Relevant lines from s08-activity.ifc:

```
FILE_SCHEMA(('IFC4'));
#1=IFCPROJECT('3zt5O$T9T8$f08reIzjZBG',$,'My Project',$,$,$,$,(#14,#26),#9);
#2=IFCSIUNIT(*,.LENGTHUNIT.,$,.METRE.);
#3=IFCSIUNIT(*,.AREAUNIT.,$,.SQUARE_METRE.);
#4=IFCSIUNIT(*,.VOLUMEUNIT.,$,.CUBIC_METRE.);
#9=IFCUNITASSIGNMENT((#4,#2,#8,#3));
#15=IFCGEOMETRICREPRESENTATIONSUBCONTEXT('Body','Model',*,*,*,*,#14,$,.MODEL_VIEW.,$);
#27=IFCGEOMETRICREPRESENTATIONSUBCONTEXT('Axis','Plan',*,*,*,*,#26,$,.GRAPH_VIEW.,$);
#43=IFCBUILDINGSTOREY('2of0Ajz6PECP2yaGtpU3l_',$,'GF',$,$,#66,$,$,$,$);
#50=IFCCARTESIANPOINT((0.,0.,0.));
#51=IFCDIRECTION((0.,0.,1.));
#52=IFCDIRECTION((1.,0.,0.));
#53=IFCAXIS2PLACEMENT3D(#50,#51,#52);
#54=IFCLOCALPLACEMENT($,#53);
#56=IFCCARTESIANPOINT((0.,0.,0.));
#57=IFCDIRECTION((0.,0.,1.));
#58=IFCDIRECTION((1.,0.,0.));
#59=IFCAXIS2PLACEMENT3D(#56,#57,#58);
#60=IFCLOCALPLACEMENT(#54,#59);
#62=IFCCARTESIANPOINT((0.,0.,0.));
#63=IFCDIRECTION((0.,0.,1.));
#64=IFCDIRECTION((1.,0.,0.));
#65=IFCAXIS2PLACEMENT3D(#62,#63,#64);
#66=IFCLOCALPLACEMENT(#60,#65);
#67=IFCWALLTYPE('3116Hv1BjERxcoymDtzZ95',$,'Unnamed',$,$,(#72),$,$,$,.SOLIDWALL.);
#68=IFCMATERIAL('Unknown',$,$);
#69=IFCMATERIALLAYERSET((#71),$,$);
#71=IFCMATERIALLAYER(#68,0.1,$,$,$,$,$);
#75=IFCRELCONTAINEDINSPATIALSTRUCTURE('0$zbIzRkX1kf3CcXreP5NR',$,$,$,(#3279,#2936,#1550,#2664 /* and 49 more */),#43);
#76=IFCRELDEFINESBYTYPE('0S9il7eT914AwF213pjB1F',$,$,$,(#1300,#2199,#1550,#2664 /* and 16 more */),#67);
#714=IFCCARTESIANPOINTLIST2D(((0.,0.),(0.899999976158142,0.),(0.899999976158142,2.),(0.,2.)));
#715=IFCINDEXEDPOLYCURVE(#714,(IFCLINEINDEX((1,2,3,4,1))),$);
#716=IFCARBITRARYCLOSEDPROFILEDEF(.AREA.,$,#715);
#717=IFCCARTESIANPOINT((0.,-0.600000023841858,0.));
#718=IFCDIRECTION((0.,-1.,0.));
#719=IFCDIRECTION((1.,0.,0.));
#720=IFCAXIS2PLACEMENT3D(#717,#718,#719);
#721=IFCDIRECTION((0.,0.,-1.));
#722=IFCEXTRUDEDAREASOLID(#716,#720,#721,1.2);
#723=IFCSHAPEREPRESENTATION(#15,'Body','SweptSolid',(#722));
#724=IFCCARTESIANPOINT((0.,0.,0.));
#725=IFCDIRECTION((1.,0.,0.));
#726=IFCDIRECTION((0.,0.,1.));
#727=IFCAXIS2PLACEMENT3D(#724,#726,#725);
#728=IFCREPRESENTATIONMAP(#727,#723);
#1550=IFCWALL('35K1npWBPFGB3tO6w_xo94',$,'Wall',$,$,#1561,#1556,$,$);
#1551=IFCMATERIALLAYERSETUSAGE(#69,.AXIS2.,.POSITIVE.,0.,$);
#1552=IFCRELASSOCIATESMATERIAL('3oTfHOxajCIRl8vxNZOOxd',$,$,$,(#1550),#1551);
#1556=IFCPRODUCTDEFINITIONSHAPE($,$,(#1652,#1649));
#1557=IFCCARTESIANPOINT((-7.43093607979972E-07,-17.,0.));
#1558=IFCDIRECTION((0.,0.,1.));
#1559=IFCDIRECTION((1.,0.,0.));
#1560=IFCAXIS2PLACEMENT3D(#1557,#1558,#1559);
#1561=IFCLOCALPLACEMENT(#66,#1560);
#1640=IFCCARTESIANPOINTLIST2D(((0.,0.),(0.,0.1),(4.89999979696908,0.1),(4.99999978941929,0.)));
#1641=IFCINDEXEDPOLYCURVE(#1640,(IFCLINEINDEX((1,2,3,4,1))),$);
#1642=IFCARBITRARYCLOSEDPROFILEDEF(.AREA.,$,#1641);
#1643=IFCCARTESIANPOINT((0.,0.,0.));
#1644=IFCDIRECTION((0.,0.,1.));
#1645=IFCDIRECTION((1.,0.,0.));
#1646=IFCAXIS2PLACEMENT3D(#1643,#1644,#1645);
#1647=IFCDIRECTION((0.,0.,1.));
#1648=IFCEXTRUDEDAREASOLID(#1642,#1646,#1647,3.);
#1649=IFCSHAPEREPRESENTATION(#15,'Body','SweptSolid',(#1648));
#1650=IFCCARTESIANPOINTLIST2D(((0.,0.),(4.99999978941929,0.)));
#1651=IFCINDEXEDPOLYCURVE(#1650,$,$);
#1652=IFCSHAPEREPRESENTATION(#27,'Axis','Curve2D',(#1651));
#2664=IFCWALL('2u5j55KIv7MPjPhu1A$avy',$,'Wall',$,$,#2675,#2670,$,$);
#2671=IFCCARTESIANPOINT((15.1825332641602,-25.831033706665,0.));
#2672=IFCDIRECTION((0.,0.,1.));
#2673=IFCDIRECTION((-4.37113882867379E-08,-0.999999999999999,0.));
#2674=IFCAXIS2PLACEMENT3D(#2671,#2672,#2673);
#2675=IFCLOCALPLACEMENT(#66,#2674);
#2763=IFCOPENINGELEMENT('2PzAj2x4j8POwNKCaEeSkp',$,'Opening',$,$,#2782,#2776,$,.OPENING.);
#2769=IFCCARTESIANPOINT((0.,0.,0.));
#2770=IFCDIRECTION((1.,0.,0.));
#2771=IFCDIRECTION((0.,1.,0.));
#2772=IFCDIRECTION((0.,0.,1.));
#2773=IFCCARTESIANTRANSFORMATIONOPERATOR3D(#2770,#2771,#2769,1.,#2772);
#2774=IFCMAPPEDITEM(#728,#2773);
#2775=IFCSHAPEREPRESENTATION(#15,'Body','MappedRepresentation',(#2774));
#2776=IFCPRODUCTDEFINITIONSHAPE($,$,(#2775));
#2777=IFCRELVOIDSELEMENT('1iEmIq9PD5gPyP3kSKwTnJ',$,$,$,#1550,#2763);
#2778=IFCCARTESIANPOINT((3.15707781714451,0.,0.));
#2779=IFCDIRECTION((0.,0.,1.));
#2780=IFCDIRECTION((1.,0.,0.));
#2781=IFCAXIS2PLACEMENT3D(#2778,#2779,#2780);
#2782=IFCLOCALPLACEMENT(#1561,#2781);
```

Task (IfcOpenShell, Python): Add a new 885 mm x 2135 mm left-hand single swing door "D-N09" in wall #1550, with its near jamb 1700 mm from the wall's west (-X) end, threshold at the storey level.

```python
import numpy as np
import ifcopenshell
import ifcopenshell.api.feature
import ifcopenshell.api.geometry
import ifcopenshell.api.root
import ifcopenshell.api.spatial
import ifcopenshell.geom
import ifcopenshell.util.element
import ifcopenshell.util.placement
import ifcopenshell.util.representation
import ifcopenshell.util.shape
import ifcopenshell.util.unit

model = ifcopenshell.open("s08-activity.ifc")
unit_scale = ifcopenshell.util.unit.calculate_unit_scale(model)
settings = ifcopenshell.geom.settings()


def volume(element):
    """Net volume in cubic metres, openings subtracted."""
    shape = ifcopenshell.geom.create_shape(settings, element)
    return ifcopenshell.util.shape.get_volume(shape.geometry)


wall = model.by_guid("35K1npWBPFGB3tO6w_xo94")
storey = ifcopenshell.util.element.get_container(wall, ifc_class="IfcBuildingStorey")
context = ifcopenshell.util.representation.get_context(model, "Model", "Body", "MODEL_VIEW")
before = volume(wall)

width, height, from_end, sill = 0.885, 2.135, 1.7, 0.0  # metres

# The wall runs along its own X axis, and the end named is its -X end.
wall_shape = ifcopenshell.geom.create_shape(settings, wall)
x, y, z = ifcopenshell.util.shape.get_vertices(wall_shape.geometry).T
start = x.min() + from_end
face, thickness = float(y.min()), float(y.max() - y.min())
wall_matrix = ifcopenshell.util.placement.get_local_placement(wall.ObjectPlacement)
level = ifcopenshell.util.placement.get_local_placement(storey.ObjectPlacement)[2, 3]


def in_wall(x, y):
    """Placement at x, y metres in the wall's axes, at sill height."""
    matrix = wall_matrix.copy()
    matrix[:, 3] = wall_matrix @ np.array([x / unit_scale, y / unit_scale, 0.0, 1.0])
    matrix[2, 3] = level + sill / unit_scale
    return matrix


# Opening: a box that overshoots both wall faces by 50 mm.
opening = ifcopenshell.api.root.create_entity(model, ifc_class="IfcOpeningElement", predefined_type="OPENING")
box = ifcopenshell.api.geometry.add_wall_representation(
    model, context=context, length=width, height=height, thickness=thickness + 0.1
)
ifcopenshell.api.geometry.assign_representation(model, product=opening, representation=box)
ifcopenshell.api.geometry.edit_object_placement(model, product=opening, matrix=in_wall(start, face - 0.05), is_si=False)
ifcopenshell.api.feature.add_feature(model, feature=opening, element=wall)

door = ifcopenshell.api.root.create_entity(model, ifc_class="IfcDoor", name="D-N09", predefined_type="DOOR")
door.OverallWidth, door.OverallHeight = width / unit_scale, height / unit_scale
door.OperationType = "SINGLE_SWING_LEFT"
body = ifcopenshell.api.geometry.add_door_representation(
    model,
    context=context,
    overall_width=door.OverallWidth,
    overall_height=door.OverallHeight,
    operation_type="SINGLE_SWING_LEFT",
    lining_properties={"LiningDepth": thickness / unit_scale, "ThresholdDepth": thickness / unit_scale},
)
ifcopenshell.api.geometry.assign_representation(model, product=door, representation=body)
ifcopenshell.api.spatial.assign_container(model, products=[door], relating_structure=storey)
ifcopenshell.api.feature.add_filling(model, opening=opening, element=door)

# The lining spans the wall, so the door starts at the wall face.
ifcopenshell.api.geometry.edit_object_placement(model, product=door, matrix=in_wall(start, face), is_si=False)

after = volume(wall)

print(f"wall volume {before:.3f} -> {after:.3f} m3")

model.write("s08-activity_edited.ifc")
```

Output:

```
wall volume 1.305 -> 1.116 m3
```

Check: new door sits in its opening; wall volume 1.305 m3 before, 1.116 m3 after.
